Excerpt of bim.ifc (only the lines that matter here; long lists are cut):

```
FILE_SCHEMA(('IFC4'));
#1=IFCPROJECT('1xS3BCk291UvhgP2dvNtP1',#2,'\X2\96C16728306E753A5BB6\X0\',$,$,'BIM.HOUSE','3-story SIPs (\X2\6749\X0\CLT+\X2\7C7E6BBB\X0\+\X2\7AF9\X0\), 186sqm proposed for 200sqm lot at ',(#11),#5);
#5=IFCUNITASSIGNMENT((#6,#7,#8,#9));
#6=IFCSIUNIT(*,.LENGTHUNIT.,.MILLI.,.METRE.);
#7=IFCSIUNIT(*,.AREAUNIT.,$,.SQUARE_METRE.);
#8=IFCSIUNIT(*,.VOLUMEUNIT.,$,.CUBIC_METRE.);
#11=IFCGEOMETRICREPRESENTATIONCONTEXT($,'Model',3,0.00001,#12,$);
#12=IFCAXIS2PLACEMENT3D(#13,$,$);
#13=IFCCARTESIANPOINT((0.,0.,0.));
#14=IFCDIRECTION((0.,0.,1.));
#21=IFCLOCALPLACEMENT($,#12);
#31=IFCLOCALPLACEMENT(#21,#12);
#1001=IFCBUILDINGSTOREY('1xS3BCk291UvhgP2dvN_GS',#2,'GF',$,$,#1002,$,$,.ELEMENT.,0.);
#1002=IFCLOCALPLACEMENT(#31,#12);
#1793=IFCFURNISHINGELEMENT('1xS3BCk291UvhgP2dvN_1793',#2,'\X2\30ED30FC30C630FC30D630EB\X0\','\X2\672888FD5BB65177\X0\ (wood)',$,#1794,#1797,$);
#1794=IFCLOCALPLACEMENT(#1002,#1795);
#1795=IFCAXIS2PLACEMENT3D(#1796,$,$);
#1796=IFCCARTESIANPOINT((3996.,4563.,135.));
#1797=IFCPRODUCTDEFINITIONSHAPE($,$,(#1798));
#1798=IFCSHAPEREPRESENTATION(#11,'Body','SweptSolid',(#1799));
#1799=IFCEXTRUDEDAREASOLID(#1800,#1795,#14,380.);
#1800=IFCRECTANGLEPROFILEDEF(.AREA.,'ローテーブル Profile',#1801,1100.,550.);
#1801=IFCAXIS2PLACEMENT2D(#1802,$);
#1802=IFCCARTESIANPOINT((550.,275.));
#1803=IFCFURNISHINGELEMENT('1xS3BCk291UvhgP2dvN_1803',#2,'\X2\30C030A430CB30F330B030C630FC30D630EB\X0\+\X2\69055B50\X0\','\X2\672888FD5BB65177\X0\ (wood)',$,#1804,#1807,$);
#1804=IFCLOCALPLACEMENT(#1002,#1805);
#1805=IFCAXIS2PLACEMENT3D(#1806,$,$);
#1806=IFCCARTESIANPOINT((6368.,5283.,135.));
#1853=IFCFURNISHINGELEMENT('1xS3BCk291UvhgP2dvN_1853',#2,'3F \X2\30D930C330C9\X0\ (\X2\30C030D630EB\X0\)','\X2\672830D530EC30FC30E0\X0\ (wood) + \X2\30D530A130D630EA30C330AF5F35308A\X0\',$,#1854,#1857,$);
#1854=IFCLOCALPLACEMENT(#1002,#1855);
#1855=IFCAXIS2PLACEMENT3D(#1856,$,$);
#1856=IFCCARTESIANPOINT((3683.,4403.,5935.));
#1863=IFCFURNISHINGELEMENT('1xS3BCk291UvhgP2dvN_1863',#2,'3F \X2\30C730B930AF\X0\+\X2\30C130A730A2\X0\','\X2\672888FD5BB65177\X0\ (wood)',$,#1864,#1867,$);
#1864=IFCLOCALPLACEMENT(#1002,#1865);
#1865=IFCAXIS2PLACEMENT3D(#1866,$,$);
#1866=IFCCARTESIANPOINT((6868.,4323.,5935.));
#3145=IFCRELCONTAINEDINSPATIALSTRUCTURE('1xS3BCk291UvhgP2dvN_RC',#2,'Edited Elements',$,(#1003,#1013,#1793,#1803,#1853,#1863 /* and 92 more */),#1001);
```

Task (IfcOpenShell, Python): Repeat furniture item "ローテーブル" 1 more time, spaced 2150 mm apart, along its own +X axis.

```python
import ifcopenshell
import ifcopenshell.api.geometry
import ifcopenshell.api.root
import ifcopenshell.util.element
import ifcopenshell.util.placement

model = ifcopenshell.open("bim.ifc")


def reuse_history(source, copy):
    """copy_class also copies each property set's owner history, people and application; keep the originals."""
    for rel in copy.IsDefinedBy:
        if rel.is_a("IfcRelDefinesByProperties") and (history := rel.RelatingPropertyDefinition.OwnerHistory):
            rel.RelatingPropertyDefinition.OwnerHistory = source.OwnerHistory
            ifcopenshell.util.element.remove_deep2(model, history)


source = model.by_guid("1xS3BCk291UvhgP2dvN_1793")
base = ifcopenshell.util.placement.get_local_placement(source.ObjectPlacement)
step = base[:3, 0] * 2150.0

for i in range(1, 2):
    copy = ifcopenshell.api.root.copy_class(model, product=source)
    copy.Representation = ifcopenshell.util.element.copy_deep(
        model, source.Representation, exclude=["IfcGeometricRepresentationContext", "IfcRepresentationMap"]
    )
    reuse_history(source, copy)
    matrix = base.copy()
    matrix[:3, 3] += i * step
    print("added at", matrix[:3, 3].round(3) + 0.0)
    ifcopenshell.api.geometry.edit_object_placement(model, product=copy, matrix=matrix, is_si=False)

model.write("bim_edited.ifc")
```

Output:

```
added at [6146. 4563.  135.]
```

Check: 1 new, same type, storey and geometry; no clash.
